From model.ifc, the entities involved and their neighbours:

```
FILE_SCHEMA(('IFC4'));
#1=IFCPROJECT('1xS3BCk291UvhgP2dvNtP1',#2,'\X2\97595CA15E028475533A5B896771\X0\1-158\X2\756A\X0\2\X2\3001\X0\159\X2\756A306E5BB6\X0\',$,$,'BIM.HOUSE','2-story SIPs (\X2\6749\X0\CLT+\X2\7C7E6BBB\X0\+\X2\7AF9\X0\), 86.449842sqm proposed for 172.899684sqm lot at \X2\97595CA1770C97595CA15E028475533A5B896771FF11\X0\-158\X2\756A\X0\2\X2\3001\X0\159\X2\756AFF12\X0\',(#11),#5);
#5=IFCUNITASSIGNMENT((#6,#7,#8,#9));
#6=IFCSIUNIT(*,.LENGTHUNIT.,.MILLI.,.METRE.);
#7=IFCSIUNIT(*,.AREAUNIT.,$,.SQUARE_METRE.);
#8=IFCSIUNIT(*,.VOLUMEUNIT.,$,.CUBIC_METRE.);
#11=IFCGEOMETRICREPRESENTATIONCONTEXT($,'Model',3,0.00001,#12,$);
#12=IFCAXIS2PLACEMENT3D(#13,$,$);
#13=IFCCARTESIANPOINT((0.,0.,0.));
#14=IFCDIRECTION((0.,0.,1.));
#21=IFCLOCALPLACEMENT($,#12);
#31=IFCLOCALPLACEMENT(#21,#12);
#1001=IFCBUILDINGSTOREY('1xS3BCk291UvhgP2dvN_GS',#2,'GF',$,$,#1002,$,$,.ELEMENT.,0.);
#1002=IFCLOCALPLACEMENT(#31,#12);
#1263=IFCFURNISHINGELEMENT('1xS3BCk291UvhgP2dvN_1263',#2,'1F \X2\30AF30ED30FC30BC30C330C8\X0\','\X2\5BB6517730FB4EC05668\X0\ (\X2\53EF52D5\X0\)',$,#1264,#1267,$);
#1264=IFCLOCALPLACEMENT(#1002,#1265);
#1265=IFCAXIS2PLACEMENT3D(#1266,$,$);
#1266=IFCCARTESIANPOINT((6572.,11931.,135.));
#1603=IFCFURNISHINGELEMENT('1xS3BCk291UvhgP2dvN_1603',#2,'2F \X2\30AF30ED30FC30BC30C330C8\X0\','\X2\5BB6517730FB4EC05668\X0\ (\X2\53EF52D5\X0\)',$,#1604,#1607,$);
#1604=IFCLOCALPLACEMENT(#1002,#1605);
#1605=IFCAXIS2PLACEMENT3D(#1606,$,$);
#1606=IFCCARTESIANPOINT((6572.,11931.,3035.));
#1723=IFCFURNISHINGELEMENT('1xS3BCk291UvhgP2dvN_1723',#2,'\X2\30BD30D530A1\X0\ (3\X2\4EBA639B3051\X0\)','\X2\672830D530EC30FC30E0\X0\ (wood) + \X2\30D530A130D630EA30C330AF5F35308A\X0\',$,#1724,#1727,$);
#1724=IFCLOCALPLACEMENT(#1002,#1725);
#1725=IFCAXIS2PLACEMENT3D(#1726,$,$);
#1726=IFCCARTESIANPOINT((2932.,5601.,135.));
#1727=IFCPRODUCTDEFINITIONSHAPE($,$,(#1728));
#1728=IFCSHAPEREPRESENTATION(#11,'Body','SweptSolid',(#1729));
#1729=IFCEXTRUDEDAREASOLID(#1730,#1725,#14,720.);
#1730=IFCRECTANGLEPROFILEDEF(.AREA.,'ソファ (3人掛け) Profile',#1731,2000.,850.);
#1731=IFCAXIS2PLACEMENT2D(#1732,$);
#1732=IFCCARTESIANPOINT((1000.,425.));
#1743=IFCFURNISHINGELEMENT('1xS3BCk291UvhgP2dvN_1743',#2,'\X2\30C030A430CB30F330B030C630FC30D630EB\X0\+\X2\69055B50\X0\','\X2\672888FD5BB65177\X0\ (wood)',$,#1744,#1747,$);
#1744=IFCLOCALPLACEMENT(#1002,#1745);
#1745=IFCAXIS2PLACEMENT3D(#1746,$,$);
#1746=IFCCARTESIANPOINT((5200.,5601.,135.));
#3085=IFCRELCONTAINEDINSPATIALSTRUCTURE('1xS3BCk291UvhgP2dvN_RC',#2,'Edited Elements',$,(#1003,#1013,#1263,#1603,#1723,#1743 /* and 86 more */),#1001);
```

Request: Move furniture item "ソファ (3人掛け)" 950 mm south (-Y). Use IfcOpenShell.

```python
import ifcopenshell
import ifcopenshell.api.geometry
import ifcopenshell.util.placement

model = ifcopenshell.open("model.ifc")

item = model.by_guid("1xS3BCk291UvhgP2dvN_1723")
matrix = ifcopenshell.util.placement.get_local_placement(item.ObjectPlacement)
matrix[1, 3] -= 950.0
ifcopenshell.api.geometry.edit_object_placement(model, product=item, matrix=matrix, is_si=False)

print(ifcopenshell.util.placement.get_local_placement(item.ObjectPlacement).round(3) + 0.0)

model.write("model_edited.ifc")
```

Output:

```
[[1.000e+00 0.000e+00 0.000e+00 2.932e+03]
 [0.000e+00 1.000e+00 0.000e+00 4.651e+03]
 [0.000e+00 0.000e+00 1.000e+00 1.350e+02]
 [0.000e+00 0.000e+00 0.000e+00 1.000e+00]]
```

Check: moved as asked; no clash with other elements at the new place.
